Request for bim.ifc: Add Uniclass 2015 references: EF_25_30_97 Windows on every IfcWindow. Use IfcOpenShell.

First a look at what the model holds.

```python
import ifcopenshell

model = ifcopenshell.open("bim.ifc")
print(model.schema)
print("classifications:", [c.Name for c in model.by_type("IfcClassification")])
for ifc_class in ("IfcDoor", "IfcRoof", "IfcStair", "IfcWall", "IfcWindow"):
    print(ifc_class, len(model.by_type(ifc_class)))
```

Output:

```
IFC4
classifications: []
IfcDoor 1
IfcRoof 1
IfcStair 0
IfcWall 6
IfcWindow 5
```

```python
import ifcopenshell
import ifcopenshell.api.classification

model = ifcopenshell.open("bim.ifc")

system = ifcopenshell.api.classification.add_classification(model, classification="Uniclass 2015")

codes = {
    "IfcWindow": ("EF_25_30_97", "Windows"),
}
for ifc_class, (code, name) in codes.items():
    products = model.by_type(ifc_class)
    ifcopenshell.api.classification.add_reference(
        model, products=products, classification=system, identification=code, name=name
    )
    print(code, len(products))

model.write("bim_rev.ifc")
```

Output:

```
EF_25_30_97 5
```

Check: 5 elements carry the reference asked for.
